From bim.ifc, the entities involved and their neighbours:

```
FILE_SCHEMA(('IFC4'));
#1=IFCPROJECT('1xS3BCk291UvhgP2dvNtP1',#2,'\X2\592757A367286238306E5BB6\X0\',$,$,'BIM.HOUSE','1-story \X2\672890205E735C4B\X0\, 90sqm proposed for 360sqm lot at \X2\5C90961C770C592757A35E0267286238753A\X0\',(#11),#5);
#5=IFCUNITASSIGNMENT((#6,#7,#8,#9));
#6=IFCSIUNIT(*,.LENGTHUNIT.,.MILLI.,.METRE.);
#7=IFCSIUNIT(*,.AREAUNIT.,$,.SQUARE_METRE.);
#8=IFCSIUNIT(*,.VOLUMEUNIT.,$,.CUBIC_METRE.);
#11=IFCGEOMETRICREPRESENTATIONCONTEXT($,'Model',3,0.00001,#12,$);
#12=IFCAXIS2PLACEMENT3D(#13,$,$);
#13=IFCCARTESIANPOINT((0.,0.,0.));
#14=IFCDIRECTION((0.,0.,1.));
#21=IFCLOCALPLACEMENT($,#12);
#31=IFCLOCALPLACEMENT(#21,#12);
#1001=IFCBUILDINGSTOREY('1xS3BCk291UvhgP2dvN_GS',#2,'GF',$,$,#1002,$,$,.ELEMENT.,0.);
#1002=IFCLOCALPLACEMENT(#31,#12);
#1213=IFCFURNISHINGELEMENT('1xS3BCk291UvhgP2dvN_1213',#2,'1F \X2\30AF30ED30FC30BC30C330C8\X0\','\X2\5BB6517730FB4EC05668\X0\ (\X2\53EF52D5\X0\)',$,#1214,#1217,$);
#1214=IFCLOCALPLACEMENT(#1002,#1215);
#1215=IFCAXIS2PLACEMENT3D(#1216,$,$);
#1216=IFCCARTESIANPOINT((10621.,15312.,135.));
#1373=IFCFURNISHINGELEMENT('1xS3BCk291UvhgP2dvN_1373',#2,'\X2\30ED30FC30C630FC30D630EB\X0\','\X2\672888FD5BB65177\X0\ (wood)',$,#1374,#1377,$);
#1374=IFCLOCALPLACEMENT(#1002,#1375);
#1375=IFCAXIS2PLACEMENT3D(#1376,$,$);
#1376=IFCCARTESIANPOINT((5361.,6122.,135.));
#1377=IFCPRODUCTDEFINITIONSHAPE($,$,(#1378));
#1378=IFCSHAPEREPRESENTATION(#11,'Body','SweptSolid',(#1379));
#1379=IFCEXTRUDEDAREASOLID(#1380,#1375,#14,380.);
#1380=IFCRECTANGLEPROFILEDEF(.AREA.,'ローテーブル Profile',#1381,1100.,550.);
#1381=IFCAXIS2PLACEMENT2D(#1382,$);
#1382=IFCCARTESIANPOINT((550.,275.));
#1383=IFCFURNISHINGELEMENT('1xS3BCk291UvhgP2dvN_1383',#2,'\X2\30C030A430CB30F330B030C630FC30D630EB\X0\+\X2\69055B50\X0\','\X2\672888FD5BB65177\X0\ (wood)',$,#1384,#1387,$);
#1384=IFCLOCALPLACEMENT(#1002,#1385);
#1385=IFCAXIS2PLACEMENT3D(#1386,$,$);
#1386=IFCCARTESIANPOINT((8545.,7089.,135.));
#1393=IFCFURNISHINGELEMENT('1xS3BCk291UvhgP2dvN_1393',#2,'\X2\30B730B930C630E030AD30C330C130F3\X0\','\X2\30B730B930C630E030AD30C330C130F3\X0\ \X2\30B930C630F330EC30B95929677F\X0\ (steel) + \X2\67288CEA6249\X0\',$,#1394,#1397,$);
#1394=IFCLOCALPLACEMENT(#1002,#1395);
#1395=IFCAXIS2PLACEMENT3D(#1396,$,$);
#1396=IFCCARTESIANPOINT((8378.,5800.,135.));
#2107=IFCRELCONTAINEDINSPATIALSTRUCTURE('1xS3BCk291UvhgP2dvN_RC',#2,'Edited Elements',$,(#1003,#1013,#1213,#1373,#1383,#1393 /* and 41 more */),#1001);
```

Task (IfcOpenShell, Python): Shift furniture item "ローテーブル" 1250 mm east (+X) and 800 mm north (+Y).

```python
import ifcopenshell
import ifcopenshell.api.geometry
import ifcopenshell.util.placement

model = ifcopenshell.open("bim.ifc")

item = model.by_guid("1xS3BCk291UvhgP2dvN_1373")
matrix = ifcopenshell.util.placement.get_local_placement(item.ObjectPlacement)
matrix[0, 3] += 1250.0
matrix[1, 3] += 800.0
ifcopenshell.api.geometry.edit_object_placement(model, product=item, matrix=matrix, is_si=False)

print(ifcopenshell.util.placement.get_local_placement(item.ObjectPlacement).round(3) + 0.0)

model.write("bim_rev.ifc")
```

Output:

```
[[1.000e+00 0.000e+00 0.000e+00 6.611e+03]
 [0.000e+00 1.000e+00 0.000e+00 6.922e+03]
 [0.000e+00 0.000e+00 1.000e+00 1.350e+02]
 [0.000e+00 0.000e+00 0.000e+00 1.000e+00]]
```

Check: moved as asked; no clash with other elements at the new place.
